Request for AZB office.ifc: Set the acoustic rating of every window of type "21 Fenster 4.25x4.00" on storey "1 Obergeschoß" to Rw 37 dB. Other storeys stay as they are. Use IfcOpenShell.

First a look at what the model holds.

```python
import ifcopenshell
import ifcopenshell.util.element

model = ifcopenshell.open("AZB office.ifc")
print(model.schema)
storey = next(s for s in model.by_type("IfcBuildingStorey") if s.Name == "1 Obergeschoß")
windows = [e for e in ifcopenshell.util.element.get_decomposition(storey) if e.is_a("IfcWindow")]
seen = {}
for e in windows:
    element_type = ifcopenshell.util.element.get_type(e)
    key = (element_type.Name if element_type != e and element_type else None, ifcopenshell.util.element.get_pset(e, "Pset_WindowCommon", "AcousticRating"))
    seen[key] = seen.get(key, 0) + 1
for (name, value), count in sorted(seen.items(), key=str):
    print(count, "x", name, "|", value)
```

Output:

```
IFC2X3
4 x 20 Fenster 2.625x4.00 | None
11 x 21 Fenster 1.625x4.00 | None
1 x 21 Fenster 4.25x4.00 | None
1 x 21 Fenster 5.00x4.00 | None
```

```python
import ifcopenshell
import ifcopenshell.api.pset
import ifcopenshell.util.element

model = ifcopenshell.open("AZB office.ifc")

storey = next(s for s in model.by_type("IfcBuildingStorey") if s.Name == "1 Obergeschoß")
windows = [e for e in ifcopenshell.util.element.get_decomposition(storey) if e.is_a("IfcWindow")]

count = 0
for e in windows:
    element_type = ifcopenshell.util.element.get_type(e)
    if element_type in (None, e) or element_type.Name != "21 Fenster 4.25x4.00":
        continue
    # add_pset returns the element's existing set when there is one.
    pset = ifcopenshell.api.pset.add_pset(model, product=e, name="Pset_WindowCommon")
    ifcopenshell.api.pset.edit_pset(model, pset=pset, properties={"AcousticRating": "Rw 37 dB"})
    count += 1

print(count, "windows updated")

model.write("AZB office-out.ifc")
```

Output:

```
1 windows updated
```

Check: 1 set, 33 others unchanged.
